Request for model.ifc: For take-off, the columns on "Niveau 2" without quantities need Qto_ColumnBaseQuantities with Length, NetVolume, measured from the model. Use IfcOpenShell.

First a look at what the model holds.

```python
import ifcopenshell
import ifcopenshell.util.element
import ifcopenshell.util.unit

model = ifcopenshell.open("model.ifc")
print(model.schema)
for unit_type in ("LENGTHUNIT", "AREAUNIT", "VOLUMEUNIT"):
    print(unit_type, ifcopenshell.util.unit.calculate_unit_scale(model, unit_type))
storey = next(s for s in model.by_type("IfcBuildingStorey") if s.Name == "Niveau 2")
columns = [e for e in ifcopenshell.util.element.get_decomposition(storey) if e.is_a("IfcColumn")]
for e in sorted(columns, key=lambda e: e.id()):
    print(e.id(), e.is_a(), e.Name, list(ifcopenshell.util.element.get_psets(e, qtos_only=True)), sep=" | ")
```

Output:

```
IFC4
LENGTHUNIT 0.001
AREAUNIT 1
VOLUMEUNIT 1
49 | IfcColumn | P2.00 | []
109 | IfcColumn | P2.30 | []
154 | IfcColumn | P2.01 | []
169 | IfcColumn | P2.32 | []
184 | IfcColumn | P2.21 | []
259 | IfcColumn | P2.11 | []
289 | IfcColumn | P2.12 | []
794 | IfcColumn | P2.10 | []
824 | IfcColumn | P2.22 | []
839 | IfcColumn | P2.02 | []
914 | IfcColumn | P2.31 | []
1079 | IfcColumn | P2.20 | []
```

```python
import ifcopenshell
import ifcopenshell.api.pset
import ifcopenshell.geom
import ifcopenshell.util.element
import ifcopenshell.util.shape
import ifcopenshell.util.unit

model = ifcopenshell.open("model.ifc")
unit_scale = ifcopenshell.util.unit.calculate_unit_scale(model)
volume_scale = ifcopenshell.util.unit.calculate_unit_scale(model, "VOLUMEUNIT")
settings = ifcopenshell.geom.settings()

storey = next(s for s in model.by_type("IfcBuildingStorey") if s.Name == "Niveau 2")
columns = [e for e in ifcopenshell.util.element.get_decomposition(storey) if e.is_a("IfcColumn")]

for e in sorted(columns, key=lambda e: e.id()):
    if ifcopenshell.util.element.get_psets(e, qtos_only=True, should_inherit=False):
        continue
    # Geometry comes back in metres, in the element's own axes.
    shape = ifcopenshell.geom.create_shape(settings, e)
    values = {
        "Length": ifcopenshell.util.shape.get_z(shape.geometry) / unit_scale,
        "NetVolume": ifcopenshell.util.shape.get_volume(shape.geometry) / volume_scale,
    }
    qto = ifcopenshell.api.pset.add_qto(model, product=e, name="Qto_ColumnBaseQuantities")
    ifcopenshell.api.pset.edit_qto(model, qto=qto, properties=values)
    print(e.id(), {k: round(v, 3) for k, v in values.items()})

model.write("model_updated.ifc")
```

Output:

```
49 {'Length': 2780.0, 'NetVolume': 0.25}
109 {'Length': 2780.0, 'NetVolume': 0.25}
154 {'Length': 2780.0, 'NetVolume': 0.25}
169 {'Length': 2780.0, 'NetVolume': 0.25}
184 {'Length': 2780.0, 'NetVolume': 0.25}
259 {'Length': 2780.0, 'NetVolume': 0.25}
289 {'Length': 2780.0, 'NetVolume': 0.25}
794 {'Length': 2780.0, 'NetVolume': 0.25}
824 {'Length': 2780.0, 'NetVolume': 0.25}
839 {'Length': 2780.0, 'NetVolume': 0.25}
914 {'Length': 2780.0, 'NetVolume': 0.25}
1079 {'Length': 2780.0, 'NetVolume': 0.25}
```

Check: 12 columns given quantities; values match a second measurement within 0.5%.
